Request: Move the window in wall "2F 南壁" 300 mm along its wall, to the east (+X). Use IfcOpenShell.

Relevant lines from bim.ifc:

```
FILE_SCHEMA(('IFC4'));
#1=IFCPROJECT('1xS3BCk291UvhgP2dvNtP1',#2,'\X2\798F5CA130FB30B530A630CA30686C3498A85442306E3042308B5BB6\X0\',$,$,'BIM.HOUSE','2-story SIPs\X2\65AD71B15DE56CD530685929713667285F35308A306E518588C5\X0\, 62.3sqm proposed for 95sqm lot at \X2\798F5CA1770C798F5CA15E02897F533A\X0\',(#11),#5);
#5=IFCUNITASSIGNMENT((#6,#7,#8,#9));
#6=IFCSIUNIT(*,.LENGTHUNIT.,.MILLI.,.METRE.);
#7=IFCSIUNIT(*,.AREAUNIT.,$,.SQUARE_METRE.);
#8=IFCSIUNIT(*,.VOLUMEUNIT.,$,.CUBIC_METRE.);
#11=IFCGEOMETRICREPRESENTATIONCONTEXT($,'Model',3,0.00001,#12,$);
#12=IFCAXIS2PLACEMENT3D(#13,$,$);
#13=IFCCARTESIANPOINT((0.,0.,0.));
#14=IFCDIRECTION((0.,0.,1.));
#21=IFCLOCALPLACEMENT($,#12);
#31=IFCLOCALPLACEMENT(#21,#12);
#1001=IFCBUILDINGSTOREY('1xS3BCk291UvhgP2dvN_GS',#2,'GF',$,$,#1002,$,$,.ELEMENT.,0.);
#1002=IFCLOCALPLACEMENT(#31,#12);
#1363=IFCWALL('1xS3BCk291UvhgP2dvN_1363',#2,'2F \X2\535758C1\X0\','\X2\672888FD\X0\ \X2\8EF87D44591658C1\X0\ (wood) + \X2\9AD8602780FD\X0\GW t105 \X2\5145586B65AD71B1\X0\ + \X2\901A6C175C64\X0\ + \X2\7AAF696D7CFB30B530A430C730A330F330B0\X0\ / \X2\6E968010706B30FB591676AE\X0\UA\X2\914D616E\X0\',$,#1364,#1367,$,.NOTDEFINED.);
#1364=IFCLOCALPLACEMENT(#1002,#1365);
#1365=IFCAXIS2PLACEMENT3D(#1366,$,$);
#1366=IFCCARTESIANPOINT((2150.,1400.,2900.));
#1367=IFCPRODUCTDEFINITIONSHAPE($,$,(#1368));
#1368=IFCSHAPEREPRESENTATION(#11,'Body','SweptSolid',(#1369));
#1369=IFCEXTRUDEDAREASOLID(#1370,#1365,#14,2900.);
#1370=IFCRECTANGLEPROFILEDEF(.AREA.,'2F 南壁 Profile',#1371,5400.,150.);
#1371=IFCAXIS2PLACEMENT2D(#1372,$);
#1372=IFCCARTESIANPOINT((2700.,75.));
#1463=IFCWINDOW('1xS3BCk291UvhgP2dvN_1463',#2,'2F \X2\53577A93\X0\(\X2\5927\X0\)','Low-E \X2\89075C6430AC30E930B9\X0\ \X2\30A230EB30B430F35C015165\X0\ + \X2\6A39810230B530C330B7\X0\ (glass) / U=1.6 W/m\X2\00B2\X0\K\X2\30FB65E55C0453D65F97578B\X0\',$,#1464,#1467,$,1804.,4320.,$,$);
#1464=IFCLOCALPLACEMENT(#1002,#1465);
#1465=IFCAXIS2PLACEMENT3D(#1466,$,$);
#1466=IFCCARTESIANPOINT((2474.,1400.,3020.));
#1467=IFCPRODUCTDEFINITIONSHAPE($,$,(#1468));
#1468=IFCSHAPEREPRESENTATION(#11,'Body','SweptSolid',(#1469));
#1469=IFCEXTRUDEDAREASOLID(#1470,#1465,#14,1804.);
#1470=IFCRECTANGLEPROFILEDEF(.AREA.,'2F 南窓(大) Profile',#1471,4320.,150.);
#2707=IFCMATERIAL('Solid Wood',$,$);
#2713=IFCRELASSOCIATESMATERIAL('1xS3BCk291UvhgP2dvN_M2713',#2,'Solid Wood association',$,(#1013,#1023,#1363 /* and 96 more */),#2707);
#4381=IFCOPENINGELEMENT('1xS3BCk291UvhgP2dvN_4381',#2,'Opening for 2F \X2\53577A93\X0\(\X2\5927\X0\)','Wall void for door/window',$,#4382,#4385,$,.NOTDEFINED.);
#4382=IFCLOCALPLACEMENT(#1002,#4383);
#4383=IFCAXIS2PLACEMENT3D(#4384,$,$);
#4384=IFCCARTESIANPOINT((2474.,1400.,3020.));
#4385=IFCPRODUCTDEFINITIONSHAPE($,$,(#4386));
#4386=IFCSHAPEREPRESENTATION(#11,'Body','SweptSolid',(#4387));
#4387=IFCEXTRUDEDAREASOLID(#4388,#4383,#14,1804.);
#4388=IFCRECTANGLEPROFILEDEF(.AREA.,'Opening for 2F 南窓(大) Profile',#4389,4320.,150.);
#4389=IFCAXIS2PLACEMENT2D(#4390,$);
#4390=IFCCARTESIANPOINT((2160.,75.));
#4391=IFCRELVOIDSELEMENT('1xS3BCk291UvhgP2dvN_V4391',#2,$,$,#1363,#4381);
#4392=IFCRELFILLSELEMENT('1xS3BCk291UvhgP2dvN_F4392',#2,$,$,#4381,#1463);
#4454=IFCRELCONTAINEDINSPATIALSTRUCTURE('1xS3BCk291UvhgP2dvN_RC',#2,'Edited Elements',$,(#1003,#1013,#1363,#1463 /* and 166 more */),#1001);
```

```python
import ifcopenshell
import ifcopenshell.api.geometry
import ifcopenshell.util.placement

model = ifcopenshell.open("bim.ifc")

window = model.by_guid("1xS3BCk291UvhgP2dvN_1463")
opening = window.FillsVoids[0].RelatingOpeningElement
wall = opening.VoidsElements[0].RelatingBuildingElement

wall_matrix = ifcopenshell.util.placement.get_local_placement(wall.ObjectPlacement)
shift = wall_matrix[:3, 0] * 300.0
before = ifcopenshell.util.placement.get_local_placement(window.ObjectPlacement)[:3, 3].copy()

# The window is not placed relative to its opening, so move both.
for product in (opening, window):
    matrix = ifcopenshell.util.placement.get_local_placement(product.ObjectPlacement)
    matrix[:3, 3] += shift
    ifcopenshell.api.geometry.edit_object_placement(model, product=product, matrix=matrix, is_si=False)

after = ifcopenshell.util.placement.get_local_placement(window.ObjectPlacement)[:3, 3]
print("window moved by", (after - before).round(3) + 0.0)

model.write("bim-out.ifc")
```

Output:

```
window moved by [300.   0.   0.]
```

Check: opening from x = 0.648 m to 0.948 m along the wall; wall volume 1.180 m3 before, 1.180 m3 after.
